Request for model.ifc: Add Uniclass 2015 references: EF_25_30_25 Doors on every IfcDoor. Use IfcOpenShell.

First a look at what the model holds.

```python
import ifcopenshell

model = ifcopenshell.open("model.ifc")
print(model.schema)
print("classifications:", [c.Name for c in model.by_type("IfcClassification")])
for ifc_class in ("IfcDoor", "IfcRoof", "IfcStair", "IfcWall", "IfcWindow"):
    print(ifc_class, len(model.by_type(ifc_class)))
```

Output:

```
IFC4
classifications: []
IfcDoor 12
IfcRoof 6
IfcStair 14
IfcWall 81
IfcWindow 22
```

```python
import ifcopenshell
import ifcopenshell.api.classification

model = ifcopenshell.open("model.ifc")

system = ifcopenshell.api.classification.add_classification(model, classification="Uniclass 2015")

codes = {
    "IfcDoor": ("EF_25_30_25", "Doors"),
}
for ifc_class, (code, name) in codes.items():
    products = model.by_type(ifc_class)
    ifcopenshell.api.classification.add_reference(
        model, products=products, classification=system, identification=code, name=name
    )
    print(code, len(products))

model.write("model_updated.ifc")
```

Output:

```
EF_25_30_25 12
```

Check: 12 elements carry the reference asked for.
